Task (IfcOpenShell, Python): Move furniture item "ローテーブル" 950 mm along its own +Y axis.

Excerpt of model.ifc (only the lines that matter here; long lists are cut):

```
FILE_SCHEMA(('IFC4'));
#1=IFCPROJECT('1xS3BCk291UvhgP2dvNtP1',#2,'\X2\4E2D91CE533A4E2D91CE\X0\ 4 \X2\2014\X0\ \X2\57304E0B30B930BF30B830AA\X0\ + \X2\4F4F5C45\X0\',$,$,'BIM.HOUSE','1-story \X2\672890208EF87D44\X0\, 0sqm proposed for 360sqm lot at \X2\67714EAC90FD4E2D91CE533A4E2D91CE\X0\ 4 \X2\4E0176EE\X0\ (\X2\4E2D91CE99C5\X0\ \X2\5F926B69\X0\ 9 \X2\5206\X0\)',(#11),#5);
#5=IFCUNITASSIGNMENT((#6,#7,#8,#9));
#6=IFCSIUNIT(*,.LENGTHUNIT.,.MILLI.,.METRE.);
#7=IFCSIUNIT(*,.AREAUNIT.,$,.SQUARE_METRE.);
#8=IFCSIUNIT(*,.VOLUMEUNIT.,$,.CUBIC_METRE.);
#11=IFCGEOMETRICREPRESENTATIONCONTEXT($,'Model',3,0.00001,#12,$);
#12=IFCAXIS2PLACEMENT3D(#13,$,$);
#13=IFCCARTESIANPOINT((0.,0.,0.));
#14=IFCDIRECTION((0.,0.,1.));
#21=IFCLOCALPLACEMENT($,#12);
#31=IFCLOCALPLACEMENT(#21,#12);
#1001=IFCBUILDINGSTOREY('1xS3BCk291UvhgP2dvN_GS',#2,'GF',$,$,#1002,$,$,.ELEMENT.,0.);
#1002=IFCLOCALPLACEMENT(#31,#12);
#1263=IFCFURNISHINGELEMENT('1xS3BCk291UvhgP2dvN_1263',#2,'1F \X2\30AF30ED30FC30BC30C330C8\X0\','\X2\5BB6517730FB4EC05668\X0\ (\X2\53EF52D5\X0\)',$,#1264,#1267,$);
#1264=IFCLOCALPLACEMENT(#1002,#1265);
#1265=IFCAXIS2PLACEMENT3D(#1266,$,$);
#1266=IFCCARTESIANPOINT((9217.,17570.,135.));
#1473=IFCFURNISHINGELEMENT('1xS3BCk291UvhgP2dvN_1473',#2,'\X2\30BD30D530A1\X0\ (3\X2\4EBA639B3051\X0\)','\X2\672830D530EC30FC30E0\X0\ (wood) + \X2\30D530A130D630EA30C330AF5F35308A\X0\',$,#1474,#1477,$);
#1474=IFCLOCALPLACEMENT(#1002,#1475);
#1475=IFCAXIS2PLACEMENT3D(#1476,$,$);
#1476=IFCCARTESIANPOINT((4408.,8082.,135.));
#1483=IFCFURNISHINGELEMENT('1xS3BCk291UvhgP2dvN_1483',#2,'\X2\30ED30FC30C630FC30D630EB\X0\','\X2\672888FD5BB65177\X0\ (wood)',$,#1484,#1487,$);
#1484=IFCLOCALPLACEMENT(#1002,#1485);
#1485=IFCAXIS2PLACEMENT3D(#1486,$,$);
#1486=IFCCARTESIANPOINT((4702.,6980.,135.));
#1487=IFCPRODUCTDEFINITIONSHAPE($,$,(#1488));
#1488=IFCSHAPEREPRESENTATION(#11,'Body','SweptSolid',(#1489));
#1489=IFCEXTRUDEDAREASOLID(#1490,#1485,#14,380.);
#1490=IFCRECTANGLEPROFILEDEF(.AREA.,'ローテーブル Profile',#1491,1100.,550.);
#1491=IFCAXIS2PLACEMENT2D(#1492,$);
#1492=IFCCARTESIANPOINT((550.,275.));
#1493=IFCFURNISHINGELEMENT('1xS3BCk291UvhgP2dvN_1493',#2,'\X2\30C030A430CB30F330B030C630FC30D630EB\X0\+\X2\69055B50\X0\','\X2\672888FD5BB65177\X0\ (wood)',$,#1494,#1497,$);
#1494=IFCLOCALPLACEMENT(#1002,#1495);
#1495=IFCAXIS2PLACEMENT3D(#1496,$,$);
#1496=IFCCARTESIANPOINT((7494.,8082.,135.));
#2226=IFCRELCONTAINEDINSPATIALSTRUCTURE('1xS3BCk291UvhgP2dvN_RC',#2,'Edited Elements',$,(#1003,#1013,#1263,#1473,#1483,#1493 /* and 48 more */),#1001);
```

```python
import ifcopenshell
import ifcopenshell.api.geometry
import ifcopenshell.util.placement
import ifcopenshell.util.unit

model = ifcopenshell.open("model.ifc")
unit_scale = ifcopenshell.util.unit.calculate_unit_scale(model)

item = model.by_guid("1xS3BCk291UvhgP2dvN_1483")
matrix = ifcopenshell.util.placement.get_local_placement(item.ObjectPlacement)
matrix[:3, 3] += matrix[:3, 1] * 0.95 / unit_scale
ifcopenshell.api.geometry.edit_object_placement(model, product=item, matrix=matrix, is_si=False)

print(ifcopenshell.util.placement.get_local_placement(item.ObjectPlacement).round(3) + 0.0)

model.write("model_v2.ifc")
```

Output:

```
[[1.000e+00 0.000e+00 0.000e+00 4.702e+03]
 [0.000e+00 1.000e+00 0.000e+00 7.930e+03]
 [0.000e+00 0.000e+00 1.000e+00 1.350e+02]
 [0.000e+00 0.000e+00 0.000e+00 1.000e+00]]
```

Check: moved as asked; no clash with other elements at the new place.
